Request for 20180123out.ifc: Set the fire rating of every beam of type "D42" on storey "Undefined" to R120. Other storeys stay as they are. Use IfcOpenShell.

First a look at what the model holds.

```python
import ifcopenshell
import ifcopenshell.util.element

model = ifcopenshell.open("20180123out.ifc")
print(model.schema)
storey = next(s for s in model.by_type("IfcBuildingStorey") if s.Name == "Undefined")
beams = [e for e in ifcopenshell.util.element.get_decomposition(storey) if e.is_a("IfcBeam")]
seen = {}
for e in beams:
    element_type = ifcopenshell.util.element.get_type(e)
    key = (element_type.Name if element_type != e and element_type else None, ifcopenshell.util.element.get_pset(e, "Pset_BeamCommon", "FireRating"))
    seen[key] = seen.get(key, 0) + 1
for (name, value), count in sorted(seen.items(), key=str):
    print(count, "x", name, "|", value)
```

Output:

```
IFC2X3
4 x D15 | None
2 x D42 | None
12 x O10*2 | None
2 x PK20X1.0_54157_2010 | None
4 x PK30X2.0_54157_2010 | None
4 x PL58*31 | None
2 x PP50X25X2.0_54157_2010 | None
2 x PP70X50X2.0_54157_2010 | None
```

```python
import ifcopenshell
import ifcopenshell.api.pset
import ifcopenshell.util.element

model = ifcopenshell.open("20180123out.ifc")

storey = next(s for s in model.by_type("IfcBuildingStorey") if s.Name == "Undefined")
beams = [e for e in ifcopenshell.util.element.get_decomposition(storey) if e.is_a("IfcBeam")]

count = 0
for e in beams:
    element_type = ifcopenshell.util.element.get_type(e)
    if element_type in (None, e) or element_type.Name != "D42":
        continue
    found = ifcopenshell.util.element.get_pset(e, "Pset_BeamCommon", should_inherit=False)
    if found:
        pset = model.by_id(found["id"])
        if len(ifcopenshell.util.element.get_elements_by_pset(pset)) > 1:
            pset = ifcopenshell.api.pset.unshare_pset(model, products=[e], pset=pset)[0]
    else:
        pset = ifcopenshell.api.pset.add_pset(model, product=e, name="Pset_BeamCommon")
    ifcopenshell.api.pset.edit_pset(model, pset=pset, properties={"FireRating": "R120"})
    count += 1

print(count, "beams updated")

model.write("20180123out_updated.ifc")
```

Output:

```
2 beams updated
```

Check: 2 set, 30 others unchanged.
